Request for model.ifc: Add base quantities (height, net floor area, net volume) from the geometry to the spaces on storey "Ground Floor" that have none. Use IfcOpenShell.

First a look at what the model holds.

```python
import ifcopenshell
import ifcopenshell.util.element
import ifcopenshell.util.unit

model = ifcopenshell.open("model.ifc")
print(model.schema)
for unit_type in ("LENGTHUNIT", "AREAUNIT", "VOLUMEUNIT"):
    print(unit_type, ifcopenshell.util.unit.calculate_unit_scale(model, unit_type))
storey = next(s for s in model.by_type("IfcBuildingStorey") if s.Name == "Ground Floor")
spaces = [e for e in ifcopenshell.util.element.get_decomposition(storey) if e.is_a("IfcSpace")]
for e in sorted(spaces, key=lambda e: e.id()):
    print(e.id(), e.is_a(), e.Name, list(ifcopenshell.util.element.get_psets(e, qtos_only=True)), sep=" | ")
```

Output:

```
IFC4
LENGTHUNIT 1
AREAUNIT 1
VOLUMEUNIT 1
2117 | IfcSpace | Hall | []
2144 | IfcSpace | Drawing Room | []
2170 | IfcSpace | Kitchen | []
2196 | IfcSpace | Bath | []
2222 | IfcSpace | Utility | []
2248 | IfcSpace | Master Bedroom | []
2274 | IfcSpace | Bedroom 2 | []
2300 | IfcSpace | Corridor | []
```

```python
import ifcopenshell
import ifcopenshell.api.pset
import ifcopenshell.geom
import ifcopenshell.util.element
import ifcopenshell.util.shape
import ifcopenshell.util.unit

model = ifcopenshell.open("model.ifc")
unit_scale = ifcopenshell.util.unit.calculate_unit_scale(model)
area_scale = ifcopenshell.util.unit.calculate_unit_scale(model, "AREAUNIT")
volume_scale = ifcopenshell.util.unit.calculate_unit_scale(model, "VOLUMEUNIT")
settings = ifcopenshell.geom.settings()

storey = next(s for s in model.by_type("IfcBuildingStorey") if s.Name == "Ground Floor")
spaces = [e for e in ifcopenshell.util.element.get_decomposition(storey) if e.is_a("IfcSpace")]

for e in sorted(spaces, key=lambda e: e.id()):
    if ifcopenshell.util.element.get_psets(e, qtos_only=True, should_inherit=False):
        continue
    # Geometry comes back in metres, in the element's own axes.
    shape = ifcopenshell.geom.create_shape(settings, e)
    values = {
        "Height": ifcopenshell.util.shape.get_z(shape.geometry) / unit_scale,
        "NetFloorArea": ifcopenshell.util.shape.get_footprint_area(shape.geometry) / area_scale,
        "NetVolume": ifcopenshell.util.shape.get_volume(shape.geometry) / volume_scale,
    }
    qto = ifcopenshell.api.pset.add_qto(model, product=e, name="Qto_SpaceBaseQuantities")
    ifcopenshell.api.pset.edit_qto(model, qto=qto, properties=values)
    print(e.id(), {k: round(v, 3) for k, v in values.items()})

model.write("model_v2.ifc")
```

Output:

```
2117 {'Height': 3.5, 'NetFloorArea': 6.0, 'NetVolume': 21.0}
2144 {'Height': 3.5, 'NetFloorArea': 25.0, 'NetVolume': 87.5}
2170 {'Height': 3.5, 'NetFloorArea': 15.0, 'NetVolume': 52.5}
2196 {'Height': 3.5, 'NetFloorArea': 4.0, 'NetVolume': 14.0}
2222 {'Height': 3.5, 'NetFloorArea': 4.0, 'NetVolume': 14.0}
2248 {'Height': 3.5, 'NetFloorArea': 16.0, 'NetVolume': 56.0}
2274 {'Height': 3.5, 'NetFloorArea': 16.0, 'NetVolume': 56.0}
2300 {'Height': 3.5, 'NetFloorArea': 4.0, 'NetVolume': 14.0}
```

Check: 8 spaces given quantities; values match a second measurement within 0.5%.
